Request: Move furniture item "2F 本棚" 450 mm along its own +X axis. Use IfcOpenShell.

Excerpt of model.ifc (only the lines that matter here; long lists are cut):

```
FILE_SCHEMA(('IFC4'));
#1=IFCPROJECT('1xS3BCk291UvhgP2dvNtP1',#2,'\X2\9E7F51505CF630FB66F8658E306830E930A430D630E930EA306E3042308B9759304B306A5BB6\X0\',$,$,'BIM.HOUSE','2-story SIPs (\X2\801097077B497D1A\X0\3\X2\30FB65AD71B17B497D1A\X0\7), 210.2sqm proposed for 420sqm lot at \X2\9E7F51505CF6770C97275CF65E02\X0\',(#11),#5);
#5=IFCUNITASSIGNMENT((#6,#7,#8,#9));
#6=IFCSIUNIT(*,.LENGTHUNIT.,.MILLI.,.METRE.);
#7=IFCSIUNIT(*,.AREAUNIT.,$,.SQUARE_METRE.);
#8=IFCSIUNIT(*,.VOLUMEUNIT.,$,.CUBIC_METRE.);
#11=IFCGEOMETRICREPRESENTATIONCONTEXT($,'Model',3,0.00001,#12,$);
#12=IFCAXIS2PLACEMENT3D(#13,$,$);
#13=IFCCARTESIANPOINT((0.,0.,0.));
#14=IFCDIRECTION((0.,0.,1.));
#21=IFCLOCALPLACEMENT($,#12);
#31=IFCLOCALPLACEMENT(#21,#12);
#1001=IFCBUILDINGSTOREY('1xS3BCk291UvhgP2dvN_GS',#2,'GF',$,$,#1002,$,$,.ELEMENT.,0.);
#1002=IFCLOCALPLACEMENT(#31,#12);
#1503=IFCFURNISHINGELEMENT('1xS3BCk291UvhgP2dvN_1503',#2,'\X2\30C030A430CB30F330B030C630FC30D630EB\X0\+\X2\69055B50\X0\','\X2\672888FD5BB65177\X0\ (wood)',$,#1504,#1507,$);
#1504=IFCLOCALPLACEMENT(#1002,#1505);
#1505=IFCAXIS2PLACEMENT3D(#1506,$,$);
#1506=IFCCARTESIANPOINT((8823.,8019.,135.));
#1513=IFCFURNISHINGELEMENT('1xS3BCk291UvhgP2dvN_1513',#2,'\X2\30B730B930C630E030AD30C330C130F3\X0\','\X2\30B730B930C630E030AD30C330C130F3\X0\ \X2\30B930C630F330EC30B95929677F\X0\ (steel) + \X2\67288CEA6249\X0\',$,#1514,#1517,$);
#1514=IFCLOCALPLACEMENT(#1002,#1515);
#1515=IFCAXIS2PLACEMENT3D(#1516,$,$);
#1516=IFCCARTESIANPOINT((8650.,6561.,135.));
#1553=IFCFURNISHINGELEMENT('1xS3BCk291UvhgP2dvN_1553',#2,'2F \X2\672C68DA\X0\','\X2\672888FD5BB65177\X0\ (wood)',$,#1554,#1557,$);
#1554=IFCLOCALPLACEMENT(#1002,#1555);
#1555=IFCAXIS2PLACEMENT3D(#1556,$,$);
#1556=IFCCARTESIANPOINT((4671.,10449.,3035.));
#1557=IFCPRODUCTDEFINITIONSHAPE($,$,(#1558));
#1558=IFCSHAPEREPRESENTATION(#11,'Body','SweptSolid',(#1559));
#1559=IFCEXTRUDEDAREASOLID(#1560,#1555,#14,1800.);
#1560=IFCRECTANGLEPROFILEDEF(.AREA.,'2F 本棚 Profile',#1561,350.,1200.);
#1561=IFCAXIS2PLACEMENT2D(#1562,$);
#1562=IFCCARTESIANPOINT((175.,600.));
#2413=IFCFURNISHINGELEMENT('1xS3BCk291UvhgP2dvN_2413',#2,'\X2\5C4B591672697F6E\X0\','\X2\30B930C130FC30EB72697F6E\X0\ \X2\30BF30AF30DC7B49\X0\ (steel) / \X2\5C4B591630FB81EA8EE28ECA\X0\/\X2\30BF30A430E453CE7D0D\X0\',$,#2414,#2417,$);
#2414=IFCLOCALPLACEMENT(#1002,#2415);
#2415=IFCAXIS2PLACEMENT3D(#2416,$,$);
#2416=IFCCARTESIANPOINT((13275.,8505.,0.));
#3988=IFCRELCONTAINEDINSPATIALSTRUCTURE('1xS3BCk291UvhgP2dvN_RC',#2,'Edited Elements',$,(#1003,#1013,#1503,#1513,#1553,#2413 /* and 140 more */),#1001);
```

```python
import ifcopenshell
import ifcopenshell.api.geometry
import ifcopenshell.util.placement
import ifcopenshell.util.unit

model = ifcopenshell.open("model.ifc")
unit_scale = ifcopenshell.util.unit.calculate_unit_scale(model)

item = model.by_id(1553)
matrix = ifcopenshell.util.placement.get_local_placement(item.ObjectPlacement)
matrix[:3, 3] += matrix[:3, 0] * 0.45 / unit_scale
ifcopenshell.api.geometry.edit_object_placement(model, product=item, matrix=matrix, is_si=False)

print(ifcopenshell.util.placement.get_local_placement(item.ObjectPlacement).round(3) + 0.0)

model.write("model-out.ifc")
```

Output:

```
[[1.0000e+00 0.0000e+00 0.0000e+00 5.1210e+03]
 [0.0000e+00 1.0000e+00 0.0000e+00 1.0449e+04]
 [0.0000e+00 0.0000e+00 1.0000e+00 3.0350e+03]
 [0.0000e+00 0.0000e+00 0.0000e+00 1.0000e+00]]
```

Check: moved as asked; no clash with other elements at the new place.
